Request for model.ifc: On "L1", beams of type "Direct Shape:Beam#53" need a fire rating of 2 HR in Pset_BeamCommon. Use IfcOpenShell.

First a look at what the model holds.

```python
import ifcopenshell
import ifcopenshell.util.element

model = ifcopenshell.open("model.ifc")
print(model.schema)
storey = next(s for s in model.by_type("IfcBuildingStorey") if s.Name == "L1")
beams = [e for e in ifcopenshell.util.element.get_decomposition(storey) if e.is_a("IfcBeam")]
seen = {}
for e in beams:
    element_type = ifcopenshell.util.element.get_type(e)
    key = (element_type.Name if element_type != e and element_type else None, ifcopenshell.util.element.get_pset(e, "Pset_BeamCommon", "FireRating"))
    seen[key] = seen.get(key, 0) + 1
for (name, value), count in sorted(seen.items(), key=str):
    print(count, "x", name, "|", value)
```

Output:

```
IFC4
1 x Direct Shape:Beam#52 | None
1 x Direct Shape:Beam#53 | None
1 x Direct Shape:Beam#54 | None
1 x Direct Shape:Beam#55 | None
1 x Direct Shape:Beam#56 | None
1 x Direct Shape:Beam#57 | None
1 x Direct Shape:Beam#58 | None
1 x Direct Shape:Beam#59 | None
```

```python
import ifcopenshell
import ifcopenshell.api.pset
import ifcopenshell.util.element

model = ifcopenshell.open("model.ifc")

storey = next(s for s in model.by_type("IfcBuildingStorey") if s.Name == "L1")
beams = [e for e in ifcopenshell.util.element.get_decomposition(storey) if e.is_a("IfcBeam")]

count = 0
for e in beams:
    element_type = ifcopenshell.util.element.get_type(e)
    if element_type in (None, e) or element_type.Name != "Direct Shape:Beam#53":
        continue
    # add_pset returns the element's existing set when there is one.
    pset = ifcopenshell.api.pset.add_pset(model, product=e, name="Pset_BeamCommon")
    ifcopenshell.api.pset.edit_pset(model, pset=pset, properties={"FireRating": "2 HR"})
    count += 1

print(count, "beams updated")

model.write("model_v2.ifc")
```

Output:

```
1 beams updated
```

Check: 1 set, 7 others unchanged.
